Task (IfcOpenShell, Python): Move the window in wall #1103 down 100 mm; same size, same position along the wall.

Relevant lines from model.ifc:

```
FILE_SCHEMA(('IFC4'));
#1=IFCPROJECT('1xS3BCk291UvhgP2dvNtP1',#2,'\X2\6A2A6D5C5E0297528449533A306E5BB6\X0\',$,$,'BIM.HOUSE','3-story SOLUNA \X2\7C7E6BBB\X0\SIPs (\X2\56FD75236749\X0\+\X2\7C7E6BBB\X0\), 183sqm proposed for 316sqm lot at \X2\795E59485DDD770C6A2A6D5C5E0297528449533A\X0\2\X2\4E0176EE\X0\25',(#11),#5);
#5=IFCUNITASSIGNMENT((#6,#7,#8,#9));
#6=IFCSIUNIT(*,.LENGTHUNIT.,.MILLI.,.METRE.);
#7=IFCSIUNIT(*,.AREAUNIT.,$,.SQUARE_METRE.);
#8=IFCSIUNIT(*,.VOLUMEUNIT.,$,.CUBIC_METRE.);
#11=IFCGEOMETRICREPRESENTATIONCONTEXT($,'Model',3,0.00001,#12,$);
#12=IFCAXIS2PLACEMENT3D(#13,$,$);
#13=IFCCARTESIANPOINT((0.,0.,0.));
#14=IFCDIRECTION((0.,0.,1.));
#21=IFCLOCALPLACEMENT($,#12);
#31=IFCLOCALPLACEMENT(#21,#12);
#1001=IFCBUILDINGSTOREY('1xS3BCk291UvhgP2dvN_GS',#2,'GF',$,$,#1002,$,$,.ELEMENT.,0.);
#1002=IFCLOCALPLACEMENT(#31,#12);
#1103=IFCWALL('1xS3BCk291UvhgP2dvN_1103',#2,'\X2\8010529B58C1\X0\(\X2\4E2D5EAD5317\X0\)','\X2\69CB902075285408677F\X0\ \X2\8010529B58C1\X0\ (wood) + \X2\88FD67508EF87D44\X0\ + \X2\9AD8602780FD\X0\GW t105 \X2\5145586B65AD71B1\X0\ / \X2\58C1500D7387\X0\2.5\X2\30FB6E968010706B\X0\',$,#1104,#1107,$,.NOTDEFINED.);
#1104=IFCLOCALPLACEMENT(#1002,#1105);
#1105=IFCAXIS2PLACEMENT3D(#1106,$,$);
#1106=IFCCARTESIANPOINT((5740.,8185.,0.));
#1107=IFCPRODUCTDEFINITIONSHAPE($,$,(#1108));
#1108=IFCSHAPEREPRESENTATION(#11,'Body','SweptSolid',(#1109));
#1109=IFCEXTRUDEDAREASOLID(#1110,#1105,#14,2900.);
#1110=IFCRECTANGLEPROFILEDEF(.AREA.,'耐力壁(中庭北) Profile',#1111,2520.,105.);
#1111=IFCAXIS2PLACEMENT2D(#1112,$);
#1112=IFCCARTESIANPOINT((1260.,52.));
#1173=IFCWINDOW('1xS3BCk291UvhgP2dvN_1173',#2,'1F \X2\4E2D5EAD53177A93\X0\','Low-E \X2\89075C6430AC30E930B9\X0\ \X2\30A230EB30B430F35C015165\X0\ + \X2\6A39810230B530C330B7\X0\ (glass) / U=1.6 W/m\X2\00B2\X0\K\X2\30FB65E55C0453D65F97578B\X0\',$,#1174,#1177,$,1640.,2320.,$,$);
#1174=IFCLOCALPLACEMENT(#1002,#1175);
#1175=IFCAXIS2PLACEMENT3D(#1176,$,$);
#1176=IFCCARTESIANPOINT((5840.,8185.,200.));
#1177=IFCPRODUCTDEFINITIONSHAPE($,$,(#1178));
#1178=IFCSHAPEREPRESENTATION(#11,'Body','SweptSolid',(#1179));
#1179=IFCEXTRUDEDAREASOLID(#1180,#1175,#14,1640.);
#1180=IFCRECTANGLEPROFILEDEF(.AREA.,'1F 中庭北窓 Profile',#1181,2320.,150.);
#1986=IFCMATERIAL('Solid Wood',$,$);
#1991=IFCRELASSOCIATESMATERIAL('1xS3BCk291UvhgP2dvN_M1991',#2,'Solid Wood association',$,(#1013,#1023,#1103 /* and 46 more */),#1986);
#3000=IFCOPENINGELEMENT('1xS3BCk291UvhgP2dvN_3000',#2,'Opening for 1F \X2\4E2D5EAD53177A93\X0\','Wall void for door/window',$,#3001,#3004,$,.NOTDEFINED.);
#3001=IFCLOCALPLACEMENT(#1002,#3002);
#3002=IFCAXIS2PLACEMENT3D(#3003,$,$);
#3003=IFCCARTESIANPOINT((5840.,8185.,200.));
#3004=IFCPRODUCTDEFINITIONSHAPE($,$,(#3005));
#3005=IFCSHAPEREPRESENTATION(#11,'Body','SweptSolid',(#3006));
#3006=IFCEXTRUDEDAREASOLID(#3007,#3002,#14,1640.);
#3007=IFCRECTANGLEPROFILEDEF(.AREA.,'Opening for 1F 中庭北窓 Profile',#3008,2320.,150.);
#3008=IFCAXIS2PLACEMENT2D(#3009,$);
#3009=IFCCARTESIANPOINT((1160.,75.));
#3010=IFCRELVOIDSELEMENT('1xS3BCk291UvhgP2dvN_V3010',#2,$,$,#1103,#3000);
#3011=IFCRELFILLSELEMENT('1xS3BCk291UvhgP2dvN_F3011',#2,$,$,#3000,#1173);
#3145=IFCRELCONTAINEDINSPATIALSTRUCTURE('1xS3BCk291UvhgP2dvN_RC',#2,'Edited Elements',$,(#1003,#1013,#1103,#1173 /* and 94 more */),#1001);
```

```python
import numpy as np
import ifcopenshell
import ifcopenshell.api.geometry
import ifcopenshell.util.placement
import ifcopenshell.util.unit

model = ifcopenshell.open("model.ifc")
unit_scale = ifcopenshell.util.unit.calculate_unit_scale(model)

window = model.by_id(1173)
opening = window.FillsVoids[0].RelatingOpeningElement
dz = -100.0

shift = np.array([0.0, 0.0, dz])
# The window is not placed relative to its opening, so move both.
for product in (opening, window):
    matrix = ifcopenshell.util.placement.get_local_placement(product.ObjectPlacement)
    matrix[:3, 3] += shift
    ifcopenshell.api.geometry.edit_object_placement(model, product=product, matrix=matrix, is_si=False)

print(f"moved by {dz * unit_scale:+.3f} m")

model.write("model_v2.ifc")
```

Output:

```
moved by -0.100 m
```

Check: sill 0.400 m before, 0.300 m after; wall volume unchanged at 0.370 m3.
